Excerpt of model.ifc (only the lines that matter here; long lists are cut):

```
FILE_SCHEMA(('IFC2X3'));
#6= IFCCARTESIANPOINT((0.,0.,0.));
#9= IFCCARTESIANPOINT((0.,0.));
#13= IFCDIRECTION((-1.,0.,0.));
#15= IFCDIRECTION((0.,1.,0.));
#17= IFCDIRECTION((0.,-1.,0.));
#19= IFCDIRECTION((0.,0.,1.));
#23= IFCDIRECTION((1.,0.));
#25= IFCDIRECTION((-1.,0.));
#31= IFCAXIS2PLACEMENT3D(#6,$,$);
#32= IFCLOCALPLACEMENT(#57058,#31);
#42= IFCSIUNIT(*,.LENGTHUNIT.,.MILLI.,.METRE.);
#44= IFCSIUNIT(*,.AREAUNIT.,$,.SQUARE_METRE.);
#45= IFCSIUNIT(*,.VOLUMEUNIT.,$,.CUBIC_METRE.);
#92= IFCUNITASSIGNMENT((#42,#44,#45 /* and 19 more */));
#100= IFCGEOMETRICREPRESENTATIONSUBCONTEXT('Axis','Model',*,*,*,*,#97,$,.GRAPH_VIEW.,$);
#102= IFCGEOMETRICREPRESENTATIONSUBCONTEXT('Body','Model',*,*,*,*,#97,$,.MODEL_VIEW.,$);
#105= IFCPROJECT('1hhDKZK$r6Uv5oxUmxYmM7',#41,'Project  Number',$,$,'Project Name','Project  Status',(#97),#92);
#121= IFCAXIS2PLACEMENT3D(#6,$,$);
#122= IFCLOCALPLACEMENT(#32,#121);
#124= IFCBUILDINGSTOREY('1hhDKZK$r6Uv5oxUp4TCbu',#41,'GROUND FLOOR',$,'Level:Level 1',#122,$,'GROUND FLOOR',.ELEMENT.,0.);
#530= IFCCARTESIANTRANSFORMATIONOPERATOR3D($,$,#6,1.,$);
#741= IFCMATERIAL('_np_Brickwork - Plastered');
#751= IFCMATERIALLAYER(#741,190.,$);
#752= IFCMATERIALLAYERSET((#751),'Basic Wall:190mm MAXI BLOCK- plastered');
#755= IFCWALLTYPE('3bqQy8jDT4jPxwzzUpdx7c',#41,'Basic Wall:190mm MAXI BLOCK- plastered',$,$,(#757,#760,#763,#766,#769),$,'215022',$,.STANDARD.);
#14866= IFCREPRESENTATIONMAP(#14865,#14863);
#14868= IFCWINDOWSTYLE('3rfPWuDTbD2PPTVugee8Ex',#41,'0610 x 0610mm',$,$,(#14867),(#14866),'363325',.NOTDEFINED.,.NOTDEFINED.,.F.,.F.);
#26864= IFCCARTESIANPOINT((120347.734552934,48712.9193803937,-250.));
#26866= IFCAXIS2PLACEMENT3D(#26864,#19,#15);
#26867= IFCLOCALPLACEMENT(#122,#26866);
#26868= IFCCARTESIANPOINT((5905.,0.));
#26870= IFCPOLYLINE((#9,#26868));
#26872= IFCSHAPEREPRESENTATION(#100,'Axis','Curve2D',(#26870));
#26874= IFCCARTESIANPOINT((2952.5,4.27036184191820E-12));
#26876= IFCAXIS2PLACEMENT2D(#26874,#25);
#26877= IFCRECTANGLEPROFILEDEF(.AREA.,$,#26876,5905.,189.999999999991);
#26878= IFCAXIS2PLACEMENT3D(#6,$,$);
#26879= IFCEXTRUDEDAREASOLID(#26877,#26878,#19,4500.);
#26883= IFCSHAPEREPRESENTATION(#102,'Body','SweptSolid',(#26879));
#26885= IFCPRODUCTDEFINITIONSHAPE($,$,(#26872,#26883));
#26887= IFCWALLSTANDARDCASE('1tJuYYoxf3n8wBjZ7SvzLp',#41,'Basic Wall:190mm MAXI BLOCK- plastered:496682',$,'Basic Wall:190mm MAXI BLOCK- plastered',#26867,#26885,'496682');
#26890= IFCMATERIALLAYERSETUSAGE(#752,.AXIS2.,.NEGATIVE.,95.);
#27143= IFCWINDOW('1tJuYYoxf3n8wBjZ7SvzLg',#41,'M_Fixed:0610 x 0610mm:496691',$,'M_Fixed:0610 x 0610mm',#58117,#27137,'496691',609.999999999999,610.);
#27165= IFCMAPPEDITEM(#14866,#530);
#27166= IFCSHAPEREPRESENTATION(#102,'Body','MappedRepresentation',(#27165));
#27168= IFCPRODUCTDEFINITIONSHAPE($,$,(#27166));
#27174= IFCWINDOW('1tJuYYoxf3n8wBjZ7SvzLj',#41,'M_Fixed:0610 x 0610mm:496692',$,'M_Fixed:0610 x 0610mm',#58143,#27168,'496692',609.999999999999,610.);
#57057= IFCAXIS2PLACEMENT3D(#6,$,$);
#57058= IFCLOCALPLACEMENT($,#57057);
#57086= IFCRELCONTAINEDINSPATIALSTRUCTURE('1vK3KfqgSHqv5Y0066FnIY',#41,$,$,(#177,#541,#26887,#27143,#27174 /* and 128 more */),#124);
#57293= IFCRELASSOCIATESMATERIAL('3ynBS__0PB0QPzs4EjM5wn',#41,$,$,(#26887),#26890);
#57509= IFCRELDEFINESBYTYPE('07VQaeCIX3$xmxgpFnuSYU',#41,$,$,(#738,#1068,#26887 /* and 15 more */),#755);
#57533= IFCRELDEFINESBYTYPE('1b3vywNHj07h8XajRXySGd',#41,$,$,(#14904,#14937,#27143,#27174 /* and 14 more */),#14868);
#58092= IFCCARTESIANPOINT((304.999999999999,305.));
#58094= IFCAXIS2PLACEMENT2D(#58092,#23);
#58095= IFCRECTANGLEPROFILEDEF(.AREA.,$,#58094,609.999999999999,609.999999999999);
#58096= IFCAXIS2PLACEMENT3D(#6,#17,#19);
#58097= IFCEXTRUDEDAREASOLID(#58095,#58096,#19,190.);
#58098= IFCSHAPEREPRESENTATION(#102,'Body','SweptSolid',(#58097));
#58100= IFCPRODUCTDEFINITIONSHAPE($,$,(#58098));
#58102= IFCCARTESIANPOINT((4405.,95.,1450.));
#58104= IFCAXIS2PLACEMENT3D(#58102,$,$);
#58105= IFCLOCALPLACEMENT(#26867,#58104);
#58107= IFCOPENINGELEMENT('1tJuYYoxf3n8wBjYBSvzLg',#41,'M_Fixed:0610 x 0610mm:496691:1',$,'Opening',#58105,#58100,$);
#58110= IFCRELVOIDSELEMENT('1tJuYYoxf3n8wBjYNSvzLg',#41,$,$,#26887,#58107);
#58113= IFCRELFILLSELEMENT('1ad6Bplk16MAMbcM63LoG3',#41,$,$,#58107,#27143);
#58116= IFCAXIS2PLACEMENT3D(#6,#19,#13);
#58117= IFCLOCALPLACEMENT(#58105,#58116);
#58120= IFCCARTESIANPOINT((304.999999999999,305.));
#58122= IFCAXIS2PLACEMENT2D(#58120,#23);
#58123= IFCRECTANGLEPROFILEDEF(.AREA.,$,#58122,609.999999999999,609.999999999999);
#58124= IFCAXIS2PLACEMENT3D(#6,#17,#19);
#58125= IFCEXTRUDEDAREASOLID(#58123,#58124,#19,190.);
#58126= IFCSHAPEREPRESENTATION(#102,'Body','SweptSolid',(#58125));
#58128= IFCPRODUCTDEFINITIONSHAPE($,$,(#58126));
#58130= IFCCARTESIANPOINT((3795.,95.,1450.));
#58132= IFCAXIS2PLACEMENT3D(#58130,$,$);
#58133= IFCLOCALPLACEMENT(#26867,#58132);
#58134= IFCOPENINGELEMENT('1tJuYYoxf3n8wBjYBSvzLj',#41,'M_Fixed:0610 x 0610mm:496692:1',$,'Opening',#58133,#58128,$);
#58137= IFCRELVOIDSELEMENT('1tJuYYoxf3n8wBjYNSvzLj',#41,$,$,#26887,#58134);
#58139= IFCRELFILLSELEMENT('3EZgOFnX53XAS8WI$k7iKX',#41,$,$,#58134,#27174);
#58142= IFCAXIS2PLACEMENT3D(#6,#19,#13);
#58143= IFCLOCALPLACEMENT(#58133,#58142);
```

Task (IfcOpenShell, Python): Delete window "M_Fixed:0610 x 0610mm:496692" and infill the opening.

```python
import ifcopenshell
import ifcopenshell.api.feature
import ifcopenshell.api.root
import ifcopenshell.geom
import ifcopenshell.util.shape

model = ifcopenshell.open("model.ifc")
settings = ifcopenshell.geom.settings()


def volume(element):
    """Net volume in cubic metres, openings subtracted."""
    shape = ifcopenshell.geom.create_shape(settings, element)
    return ifcopenshell.util.shape.get_volume(shape.geometry)


window = model.by_guid("1tJuYYoxf3n8wBjZ7SvzLj")
opening = window.FillsVoids[0].RelatingOpeningElement
wall = opening.VoidsElements[0].RelatingBuildingElement
before = volume(wall)

ifcopenshell.api.root.remove_product(model, product=window)
ifcopenshell.api.feature.remove_feature(model, feature=opening)

after = volume(wall)

print(f"wall volume {before:.3f} -> {after:.3f} m3")

model.write("model_rev.ifc")
```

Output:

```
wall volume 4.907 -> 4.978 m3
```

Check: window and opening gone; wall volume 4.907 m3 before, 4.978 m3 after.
